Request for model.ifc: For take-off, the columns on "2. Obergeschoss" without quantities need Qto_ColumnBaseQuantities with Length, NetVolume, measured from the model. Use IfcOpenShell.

First a look at what the model holds.

```python
import ifcopenshell
import ifcopenshell.util.element
import ifcopenshell.util.unit

model = ifcopenshell.open("model.ifc")
print(model.schema)
for unit_type in ("LENGTHUNIT", "AREAUNIT", "VOLUMEUNIT"):
    print(unit_type, ifcopenshell.util.unit.calculate_unit_scale(model, unit_type))
storey = next(s for s in model.by_type("IfcBuildingStorey") if s.Name == "2. Obergeschoss")
columns = [e for e in ifcopenshell.util.element.get_decomposition(storey) if e.is_a("IfcColumn")]
for e in sorted(columns, key=lambda e: e.id()):
    print(e.id(), e.is_a(), e.Name, list(ifcopenshell.util.element.get_psets(e, qtos_only=True)), sep=" | ")
```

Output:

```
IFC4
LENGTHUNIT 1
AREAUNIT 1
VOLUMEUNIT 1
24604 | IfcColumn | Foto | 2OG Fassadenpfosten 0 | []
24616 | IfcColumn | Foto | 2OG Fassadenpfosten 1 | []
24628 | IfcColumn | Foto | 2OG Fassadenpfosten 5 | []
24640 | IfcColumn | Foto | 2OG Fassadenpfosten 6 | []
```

```python
import ifcopenshell
import ifcopenshell.api.pset
import ifcopenshell.geom
import ifcopenshell.util.element
import ifcopenshell.util.shape
import ifcopenshell.util.unit

model = ifcopenshell.open("model.ifc")
unit_scale = ifcopenshell.util.unit.calculate_unit_scale(model)
volume_scale = ifcopenshell.util.unit.calculate_unit_scale(model, "VOLUMEUNIT")
settings = ifcopenshell.geom.settings()

storey = next(s for s in model.by_type("IfcBuildingStorey") if s.Name == "2. Obergeschoss")
columns = [e for e in ifcopenshell.util.element.get_decomposition(storey) if e.is_a("IfcColumn")]

for e in sorted(columns, key=lambda e: e.id()):
    if ifcopenshell.util.element.get_psets(e, qtos_only=True, should_inherit=False):
        continue
    # Geometry comes back in metres, in the element's own axes.
    shape = ifcopenshell.geom.create_shape(settings, e)
    values = {
        "Length": ifcopenshell.util.shape.get_z(shape.geometry) / unit_scale,
        "NetVolume": ifcopenshell.util.shape.get_volume(shape.geometry) / volume_scale,
    }
    qto = ifcopenshell.api.pset.add_qto(model, product=e, name="Qto_ColumnBaseQuantities")
    ifcopenshell.api.pset.edit_qto(model, qto=qto, properties=values)
    print(e.id(), {k: round(v, 3) for k, v in values.items()})

model.write("model_v2.ifc")
```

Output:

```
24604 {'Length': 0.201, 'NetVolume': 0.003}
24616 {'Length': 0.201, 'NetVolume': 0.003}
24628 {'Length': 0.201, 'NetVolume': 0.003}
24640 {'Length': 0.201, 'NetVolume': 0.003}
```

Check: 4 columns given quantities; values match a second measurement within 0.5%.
